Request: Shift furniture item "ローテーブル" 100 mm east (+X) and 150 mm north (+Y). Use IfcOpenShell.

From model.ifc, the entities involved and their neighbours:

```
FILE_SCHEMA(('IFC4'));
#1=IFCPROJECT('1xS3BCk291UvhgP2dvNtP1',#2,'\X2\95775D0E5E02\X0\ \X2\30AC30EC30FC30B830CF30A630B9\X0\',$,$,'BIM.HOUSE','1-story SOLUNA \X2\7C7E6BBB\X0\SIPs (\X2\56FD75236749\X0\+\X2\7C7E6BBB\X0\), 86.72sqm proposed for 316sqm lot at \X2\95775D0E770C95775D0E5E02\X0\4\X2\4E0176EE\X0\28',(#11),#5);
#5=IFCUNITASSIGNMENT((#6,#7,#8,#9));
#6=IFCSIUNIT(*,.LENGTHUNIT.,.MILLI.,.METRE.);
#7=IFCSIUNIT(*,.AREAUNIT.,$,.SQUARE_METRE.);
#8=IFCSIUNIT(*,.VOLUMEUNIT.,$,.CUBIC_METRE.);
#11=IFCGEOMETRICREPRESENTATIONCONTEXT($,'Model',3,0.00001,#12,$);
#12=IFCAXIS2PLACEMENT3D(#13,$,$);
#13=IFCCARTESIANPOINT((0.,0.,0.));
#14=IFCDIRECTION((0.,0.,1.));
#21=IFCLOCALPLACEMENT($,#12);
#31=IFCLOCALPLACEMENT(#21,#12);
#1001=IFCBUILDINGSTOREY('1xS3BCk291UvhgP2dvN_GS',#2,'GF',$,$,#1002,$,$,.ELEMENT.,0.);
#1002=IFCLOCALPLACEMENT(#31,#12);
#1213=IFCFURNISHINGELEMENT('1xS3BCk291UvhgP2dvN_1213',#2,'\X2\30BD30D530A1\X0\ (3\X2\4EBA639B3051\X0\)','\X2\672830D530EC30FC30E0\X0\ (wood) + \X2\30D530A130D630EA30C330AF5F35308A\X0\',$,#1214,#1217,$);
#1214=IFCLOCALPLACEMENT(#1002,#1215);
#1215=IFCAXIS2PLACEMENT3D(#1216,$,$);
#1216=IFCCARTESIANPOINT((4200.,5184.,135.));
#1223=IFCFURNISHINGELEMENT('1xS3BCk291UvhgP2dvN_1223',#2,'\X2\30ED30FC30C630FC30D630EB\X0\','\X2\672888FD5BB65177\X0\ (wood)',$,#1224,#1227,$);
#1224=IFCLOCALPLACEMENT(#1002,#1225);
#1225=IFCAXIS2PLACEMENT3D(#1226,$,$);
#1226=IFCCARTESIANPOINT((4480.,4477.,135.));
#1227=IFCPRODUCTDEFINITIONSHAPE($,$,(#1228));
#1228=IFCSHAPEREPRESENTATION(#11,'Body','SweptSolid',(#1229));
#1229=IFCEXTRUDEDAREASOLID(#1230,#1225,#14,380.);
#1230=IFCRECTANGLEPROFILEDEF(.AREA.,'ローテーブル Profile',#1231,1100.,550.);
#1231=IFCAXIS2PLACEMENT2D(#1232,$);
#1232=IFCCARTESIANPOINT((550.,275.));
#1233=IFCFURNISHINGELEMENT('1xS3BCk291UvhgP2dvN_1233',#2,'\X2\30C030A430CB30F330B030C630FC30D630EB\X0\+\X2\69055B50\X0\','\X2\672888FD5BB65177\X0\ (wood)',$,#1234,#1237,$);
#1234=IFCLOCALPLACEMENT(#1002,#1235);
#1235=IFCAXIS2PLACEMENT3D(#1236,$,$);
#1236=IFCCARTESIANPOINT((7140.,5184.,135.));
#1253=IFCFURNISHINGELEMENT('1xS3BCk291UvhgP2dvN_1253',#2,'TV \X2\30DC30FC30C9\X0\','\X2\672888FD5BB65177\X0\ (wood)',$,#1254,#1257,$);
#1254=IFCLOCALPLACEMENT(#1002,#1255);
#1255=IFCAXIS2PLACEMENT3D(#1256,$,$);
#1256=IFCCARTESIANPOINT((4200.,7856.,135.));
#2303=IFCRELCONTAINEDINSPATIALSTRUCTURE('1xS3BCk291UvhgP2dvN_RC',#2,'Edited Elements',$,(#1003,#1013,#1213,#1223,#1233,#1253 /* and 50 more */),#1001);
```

```python
import ifcopenshell
import ifcopenshell.api.geometry
import ifcopenshell.util.placement
import ifcopenshell.util.unit

model = ifcopenshell.open("model.ifc")
unit_scale = ifcopenshell.util.unit.calculate_unit_scale(model)

item = model.by_guid("1xS3BCk291UvhgP2dvN_1223")
matrix = ifcopenshell.util.placement.get_local_placement(item.ObjectPlacement)
matrix[0, 3] += 0.1 / unit_scale
matrix[1, 3] += 0.15 / unit_scale
ifcopenshell.api.geometry.edit_object_placement(model, product=item, matrix=matrix, is_si=False)

print(ifcopenshell.util.placement.get_local_placement(item.ObjectPlacement).round(3) + 0.0)

model.write("model_edited.ifc")
```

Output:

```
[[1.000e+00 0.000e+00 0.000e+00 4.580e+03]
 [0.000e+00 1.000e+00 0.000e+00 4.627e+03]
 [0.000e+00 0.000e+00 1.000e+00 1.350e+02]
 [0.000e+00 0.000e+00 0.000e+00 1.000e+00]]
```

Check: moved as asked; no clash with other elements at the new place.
